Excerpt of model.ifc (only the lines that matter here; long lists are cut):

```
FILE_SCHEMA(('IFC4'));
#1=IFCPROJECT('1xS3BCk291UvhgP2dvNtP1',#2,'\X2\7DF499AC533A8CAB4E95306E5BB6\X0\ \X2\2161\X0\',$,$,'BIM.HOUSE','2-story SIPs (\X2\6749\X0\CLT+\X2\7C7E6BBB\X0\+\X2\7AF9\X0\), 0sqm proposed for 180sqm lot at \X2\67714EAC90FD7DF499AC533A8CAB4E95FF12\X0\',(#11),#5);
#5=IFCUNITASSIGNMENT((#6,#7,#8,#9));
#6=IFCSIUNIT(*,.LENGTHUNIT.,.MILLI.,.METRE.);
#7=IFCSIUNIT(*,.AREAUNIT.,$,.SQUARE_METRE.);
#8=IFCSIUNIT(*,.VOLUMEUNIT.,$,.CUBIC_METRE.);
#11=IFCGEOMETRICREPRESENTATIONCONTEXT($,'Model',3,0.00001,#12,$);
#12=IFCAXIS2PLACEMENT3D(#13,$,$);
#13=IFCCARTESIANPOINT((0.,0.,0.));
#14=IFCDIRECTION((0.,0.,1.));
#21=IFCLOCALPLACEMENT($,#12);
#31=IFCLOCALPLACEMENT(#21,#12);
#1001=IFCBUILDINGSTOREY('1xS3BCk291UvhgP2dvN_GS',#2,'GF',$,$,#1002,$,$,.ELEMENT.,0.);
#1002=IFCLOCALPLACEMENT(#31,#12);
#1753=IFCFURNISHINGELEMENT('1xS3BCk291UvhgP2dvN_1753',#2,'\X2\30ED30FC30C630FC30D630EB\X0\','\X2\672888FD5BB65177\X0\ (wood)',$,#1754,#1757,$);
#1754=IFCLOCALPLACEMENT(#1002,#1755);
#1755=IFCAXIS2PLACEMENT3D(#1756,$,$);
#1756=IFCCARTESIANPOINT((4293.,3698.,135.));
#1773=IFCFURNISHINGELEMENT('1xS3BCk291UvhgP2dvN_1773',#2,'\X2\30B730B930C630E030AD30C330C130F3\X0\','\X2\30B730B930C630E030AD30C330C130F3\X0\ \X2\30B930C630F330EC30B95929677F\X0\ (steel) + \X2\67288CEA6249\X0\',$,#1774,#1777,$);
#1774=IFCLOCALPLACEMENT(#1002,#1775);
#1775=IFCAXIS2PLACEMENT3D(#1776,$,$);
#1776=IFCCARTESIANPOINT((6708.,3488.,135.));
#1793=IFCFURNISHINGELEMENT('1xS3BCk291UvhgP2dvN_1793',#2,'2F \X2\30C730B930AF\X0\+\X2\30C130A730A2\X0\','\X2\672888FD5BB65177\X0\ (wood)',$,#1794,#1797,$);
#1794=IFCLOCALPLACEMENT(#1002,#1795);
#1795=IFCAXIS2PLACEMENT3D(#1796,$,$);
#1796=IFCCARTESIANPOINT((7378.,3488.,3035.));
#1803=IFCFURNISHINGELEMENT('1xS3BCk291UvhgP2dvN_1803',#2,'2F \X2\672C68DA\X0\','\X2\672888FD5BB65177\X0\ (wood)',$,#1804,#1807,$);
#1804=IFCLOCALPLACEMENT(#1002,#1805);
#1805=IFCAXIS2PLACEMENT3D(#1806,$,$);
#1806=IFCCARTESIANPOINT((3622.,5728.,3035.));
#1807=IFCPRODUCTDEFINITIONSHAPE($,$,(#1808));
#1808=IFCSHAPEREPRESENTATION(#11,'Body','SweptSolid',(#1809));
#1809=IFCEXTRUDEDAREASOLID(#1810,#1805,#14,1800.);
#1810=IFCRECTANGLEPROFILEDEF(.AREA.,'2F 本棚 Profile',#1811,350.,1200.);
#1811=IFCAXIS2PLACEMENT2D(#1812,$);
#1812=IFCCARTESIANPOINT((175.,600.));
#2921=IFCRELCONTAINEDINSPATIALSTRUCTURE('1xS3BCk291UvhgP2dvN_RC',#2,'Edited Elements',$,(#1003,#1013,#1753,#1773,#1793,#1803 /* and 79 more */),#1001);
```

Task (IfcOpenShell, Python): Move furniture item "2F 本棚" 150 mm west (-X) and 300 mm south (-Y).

```python
import ifcopenshell
import ifcopenshell.api.geometry
import ifcopenshell.util.placement
import ifcopenshell.util.unit

model = ifcopenshell.open("model.ifc")
unit_scale = ifcopenshell.util.unit.calculate_unit_scale(model)

item = model.by_guid("1xS3BCk291UvhgP2dvN_1803")
matrix = ifcopenshell.util.placement.get_local_placement(item.ObjectPlacement)
matrix[0, 3] -= 0.15 / unit_scale
matrix[1, 3] -= 0.3 / unit_scale
ifcopenshell.api.geometry.edit_object_placement(model, product=item, matrix=matrix, is_si=False)

print(ifcopenshell.util.placement.get_local_placement(item.ObjectPlacement).round(3) + 0.0)

model.write("model-out.ifc")
```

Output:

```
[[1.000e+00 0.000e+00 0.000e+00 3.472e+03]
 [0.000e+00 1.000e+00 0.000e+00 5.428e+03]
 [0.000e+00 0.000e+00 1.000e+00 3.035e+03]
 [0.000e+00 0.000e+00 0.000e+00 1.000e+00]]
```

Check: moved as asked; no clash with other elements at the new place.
